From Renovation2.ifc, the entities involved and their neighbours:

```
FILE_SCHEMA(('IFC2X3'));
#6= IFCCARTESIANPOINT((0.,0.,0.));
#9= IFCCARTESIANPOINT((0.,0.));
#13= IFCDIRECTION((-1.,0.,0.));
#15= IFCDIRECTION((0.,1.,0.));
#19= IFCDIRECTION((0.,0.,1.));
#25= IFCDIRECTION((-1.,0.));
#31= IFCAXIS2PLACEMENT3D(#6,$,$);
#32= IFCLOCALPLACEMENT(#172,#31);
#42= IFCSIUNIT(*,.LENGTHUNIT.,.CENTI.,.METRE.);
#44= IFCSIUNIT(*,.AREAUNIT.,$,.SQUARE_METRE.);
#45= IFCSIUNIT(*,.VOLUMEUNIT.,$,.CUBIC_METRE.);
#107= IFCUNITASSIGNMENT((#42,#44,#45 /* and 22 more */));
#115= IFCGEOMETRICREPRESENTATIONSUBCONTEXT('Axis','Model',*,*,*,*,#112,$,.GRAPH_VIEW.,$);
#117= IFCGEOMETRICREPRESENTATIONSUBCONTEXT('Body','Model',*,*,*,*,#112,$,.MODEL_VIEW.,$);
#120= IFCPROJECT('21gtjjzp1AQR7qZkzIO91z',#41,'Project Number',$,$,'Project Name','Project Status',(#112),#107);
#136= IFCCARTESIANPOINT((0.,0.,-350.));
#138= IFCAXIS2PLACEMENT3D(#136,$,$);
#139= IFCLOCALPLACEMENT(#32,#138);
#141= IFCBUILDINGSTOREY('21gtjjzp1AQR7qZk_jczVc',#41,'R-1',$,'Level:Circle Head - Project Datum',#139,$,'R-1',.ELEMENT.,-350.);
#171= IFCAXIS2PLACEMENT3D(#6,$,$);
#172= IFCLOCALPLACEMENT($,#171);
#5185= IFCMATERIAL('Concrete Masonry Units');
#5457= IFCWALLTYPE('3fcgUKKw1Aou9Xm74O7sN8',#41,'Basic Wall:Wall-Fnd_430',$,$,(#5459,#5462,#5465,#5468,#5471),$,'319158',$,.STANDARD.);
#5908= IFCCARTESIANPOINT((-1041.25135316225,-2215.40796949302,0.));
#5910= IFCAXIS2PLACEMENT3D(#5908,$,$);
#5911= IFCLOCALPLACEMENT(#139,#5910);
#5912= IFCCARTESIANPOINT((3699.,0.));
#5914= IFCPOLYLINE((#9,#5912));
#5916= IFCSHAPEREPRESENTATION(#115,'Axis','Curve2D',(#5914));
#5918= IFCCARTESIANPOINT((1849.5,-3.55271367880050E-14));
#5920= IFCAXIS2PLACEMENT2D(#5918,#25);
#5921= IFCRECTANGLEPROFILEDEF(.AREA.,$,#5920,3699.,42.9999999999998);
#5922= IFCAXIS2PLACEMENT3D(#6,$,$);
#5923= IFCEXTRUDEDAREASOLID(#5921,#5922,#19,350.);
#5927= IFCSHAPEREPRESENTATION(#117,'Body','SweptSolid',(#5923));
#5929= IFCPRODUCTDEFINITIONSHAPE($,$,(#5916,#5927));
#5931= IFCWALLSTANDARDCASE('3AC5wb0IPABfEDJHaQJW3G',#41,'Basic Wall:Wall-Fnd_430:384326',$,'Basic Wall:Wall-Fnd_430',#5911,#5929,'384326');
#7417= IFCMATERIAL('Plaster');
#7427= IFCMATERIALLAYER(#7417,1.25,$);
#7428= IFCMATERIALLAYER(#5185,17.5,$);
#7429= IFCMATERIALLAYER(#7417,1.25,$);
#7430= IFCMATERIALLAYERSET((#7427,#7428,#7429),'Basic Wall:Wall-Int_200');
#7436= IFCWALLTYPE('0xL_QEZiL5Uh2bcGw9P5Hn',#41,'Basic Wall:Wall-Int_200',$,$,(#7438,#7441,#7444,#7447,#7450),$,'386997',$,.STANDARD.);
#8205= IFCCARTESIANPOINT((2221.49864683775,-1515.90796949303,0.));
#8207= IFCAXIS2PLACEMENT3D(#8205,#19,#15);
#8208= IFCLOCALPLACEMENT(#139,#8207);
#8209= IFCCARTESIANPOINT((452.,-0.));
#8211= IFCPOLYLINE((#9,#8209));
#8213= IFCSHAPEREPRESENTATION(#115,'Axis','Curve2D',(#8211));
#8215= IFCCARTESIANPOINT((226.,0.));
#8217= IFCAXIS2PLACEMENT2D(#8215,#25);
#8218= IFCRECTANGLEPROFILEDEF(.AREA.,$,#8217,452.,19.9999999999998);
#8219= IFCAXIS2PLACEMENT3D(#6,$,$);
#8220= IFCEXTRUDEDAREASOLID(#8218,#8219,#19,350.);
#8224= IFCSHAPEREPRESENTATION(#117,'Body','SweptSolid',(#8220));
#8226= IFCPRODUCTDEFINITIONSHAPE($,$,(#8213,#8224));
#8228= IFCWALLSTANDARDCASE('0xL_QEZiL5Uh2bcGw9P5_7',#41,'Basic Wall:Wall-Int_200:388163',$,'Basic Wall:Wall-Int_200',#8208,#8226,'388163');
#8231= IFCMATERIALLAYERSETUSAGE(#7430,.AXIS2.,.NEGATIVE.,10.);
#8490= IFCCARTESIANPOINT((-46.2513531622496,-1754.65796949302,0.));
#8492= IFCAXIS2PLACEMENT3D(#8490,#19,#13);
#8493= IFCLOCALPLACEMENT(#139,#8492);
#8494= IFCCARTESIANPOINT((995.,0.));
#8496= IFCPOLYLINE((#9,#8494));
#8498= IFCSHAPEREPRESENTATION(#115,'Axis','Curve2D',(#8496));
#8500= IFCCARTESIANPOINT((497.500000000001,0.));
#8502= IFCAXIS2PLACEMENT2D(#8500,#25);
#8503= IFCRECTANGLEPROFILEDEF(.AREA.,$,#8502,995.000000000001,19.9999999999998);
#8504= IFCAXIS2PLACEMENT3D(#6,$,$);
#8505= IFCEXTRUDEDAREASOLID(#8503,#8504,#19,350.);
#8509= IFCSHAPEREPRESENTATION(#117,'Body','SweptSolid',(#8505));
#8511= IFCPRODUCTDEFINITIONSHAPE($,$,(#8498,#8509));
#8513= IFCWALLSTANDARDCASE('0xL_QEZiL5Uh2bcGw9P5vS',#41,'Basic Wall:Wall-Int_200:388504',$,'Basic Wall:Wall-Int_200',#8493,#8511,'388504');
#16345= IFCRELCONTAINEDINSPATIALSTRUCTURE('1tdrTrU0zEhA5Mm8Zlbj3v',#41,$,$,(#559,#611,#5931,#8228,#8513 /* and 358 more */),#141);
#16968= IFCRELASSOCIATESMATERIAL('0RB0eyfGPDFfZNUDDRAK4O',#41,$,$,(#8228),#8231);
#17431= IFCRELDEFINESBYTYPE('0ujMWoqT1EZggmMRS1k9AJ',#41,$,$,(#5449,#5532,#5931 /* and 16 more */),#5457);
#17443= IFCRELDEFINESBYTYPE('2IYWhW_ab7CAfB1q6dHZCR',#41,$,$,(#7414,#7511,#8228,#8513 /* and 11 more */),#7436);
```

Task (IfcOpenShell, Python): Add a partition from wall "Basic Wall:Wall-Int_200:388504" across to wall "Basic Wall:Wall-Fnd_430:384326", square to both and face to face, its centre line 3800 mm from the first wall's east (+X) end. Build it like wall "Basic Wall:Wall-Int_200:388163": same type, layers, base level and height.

```python
import numpy as np
import ifcopenshell
import ifcopenshell.api.geometry
import ifcopenshell.api.material
import ifcopenshell.api.pset
import ifcopenshell.api.root
import ifcopenshell.api.spatial
import ifcopenshell.api.type
import ifcopenshell.geom
import ifcopenshell.util.element
import ifcopenshell.util.placement
import ifcopenshell.util.representation
import ifcopenshell.util.shape
import ifcopenshell.util.unit

model = ifcopenshell.open("Renovation2.ifc")
unit_scale = ifcopenshell.util.unit.calculate_unit_scale(model)
settings = ifcopenshell.geom.settings()
settings.set("use-world-coords", True)

start_wall = model.by_guid("0xL_QEZiL5Uh2bcGw9P5vS")
end_wall = model.by_guid("3AC5wb0IPABfEDJHaQJW3G")
like = model.by_guid("0xL_QEZiL5Uh2bcGw9P5_7")
matrix = ifcopenshell.util.placement.get_local_placement(start_wall.ObjectPlacement)
matrix[:3, 3] *= unit_scale


def extent(element):
    """Bounding box in the first wall's axes, in metres."""
    shape = ifcopenshell.geom.create_shape(settings, element)
    points = (ifcopenshell.util.shape.get_vertices(shape.geometry) - matrix[:3, 3]) @ matrix[:3, :3]
    return points.min(axis=0), points.max(axis=0)


y_start = extent(start_wall)[1][1]
y_end = extent(end_wall)[0][1]
like_min, like_max = extent(like)
length, height = float(abs(y_end - y_start)), float(like_max[2] - like_min[2])
layer_set = ifcopenshell.util.element.get_material(like, should_skip_usage=True)
thickness = sum(layer.LayerThickness for layer in layer_set.MaterialLayers) * unit_scale

wall = ifcopenshell.api.root.create_entity(model, ifc_class="IfcWallStandardCase", name="New partition")
storey = ifcopenshell.util.element.get_container(like)
ifcopenshell.api.spatial.assign_container(model, products=[wall], relating_structure=storey)
ifcopenshell.api.type.assign_type(
    model, related_objects=[wall], relating_type=ifcopenshell.util.element.get_type(like), should_map_representations=False
)
rel = ifcopenshell.api.material.assign_material(
    model, products=[wall], type="IfcMaterialLayerSetUsage", material=layer_set
)
rel.RelatingMaterial.OffsetFromReferenceLine = -thickness / 2 / unit_scale
pset = ifcopenshell.api.pset.add_pset(model, product=wall, name="Pset_WallCommon")
ifcopenshell.api.pset.edit_pset(model, pset=pset, properties={"IsExternal": False, "LoadBearing": False})

# The axis runs down the middle of the wall.
axis = ifcopenshell.api.geometry.add_axis_representation(
    model, context=ifcopenshell.util.representation.get_context(model, "Model", "Axis"), axis=[(0.0, 0.0), (length, 0.0)]
)
body = ifcopenshell.api.geometry.add_wall_representation(
    model,
    context=ifcopenshell.util.representation.get_context(model, "Model", "Body", "MODEL_VIEW"),
    length=length,
    height=height,
    thickness=thickness,
    offset=-thickness / 2,
)
for representation in (axis, body):
    ifcopenshell.api.geometry.assign_representation(model, product=wall, representation=representation)

placement = matrix @ ifcopenshell.util.placement.rotation(90, "Z")
placement[:, 3] = matrix @ np.array([extent(start_wall)[0][0] + 3.8, y_start, like_min[2], 1.0])
ifcopenshell.api.geometry.edit_object_placement(model, product=wall, matrix=placement)

print(f"partition {length:.3f} m long, {height:.3f} m high, {thickness:.3f} m thick")

model.write("Renovation2_rev.ifc")
```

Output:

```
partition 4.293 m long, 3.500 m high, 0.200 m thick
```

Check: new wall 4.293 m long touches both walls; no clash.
